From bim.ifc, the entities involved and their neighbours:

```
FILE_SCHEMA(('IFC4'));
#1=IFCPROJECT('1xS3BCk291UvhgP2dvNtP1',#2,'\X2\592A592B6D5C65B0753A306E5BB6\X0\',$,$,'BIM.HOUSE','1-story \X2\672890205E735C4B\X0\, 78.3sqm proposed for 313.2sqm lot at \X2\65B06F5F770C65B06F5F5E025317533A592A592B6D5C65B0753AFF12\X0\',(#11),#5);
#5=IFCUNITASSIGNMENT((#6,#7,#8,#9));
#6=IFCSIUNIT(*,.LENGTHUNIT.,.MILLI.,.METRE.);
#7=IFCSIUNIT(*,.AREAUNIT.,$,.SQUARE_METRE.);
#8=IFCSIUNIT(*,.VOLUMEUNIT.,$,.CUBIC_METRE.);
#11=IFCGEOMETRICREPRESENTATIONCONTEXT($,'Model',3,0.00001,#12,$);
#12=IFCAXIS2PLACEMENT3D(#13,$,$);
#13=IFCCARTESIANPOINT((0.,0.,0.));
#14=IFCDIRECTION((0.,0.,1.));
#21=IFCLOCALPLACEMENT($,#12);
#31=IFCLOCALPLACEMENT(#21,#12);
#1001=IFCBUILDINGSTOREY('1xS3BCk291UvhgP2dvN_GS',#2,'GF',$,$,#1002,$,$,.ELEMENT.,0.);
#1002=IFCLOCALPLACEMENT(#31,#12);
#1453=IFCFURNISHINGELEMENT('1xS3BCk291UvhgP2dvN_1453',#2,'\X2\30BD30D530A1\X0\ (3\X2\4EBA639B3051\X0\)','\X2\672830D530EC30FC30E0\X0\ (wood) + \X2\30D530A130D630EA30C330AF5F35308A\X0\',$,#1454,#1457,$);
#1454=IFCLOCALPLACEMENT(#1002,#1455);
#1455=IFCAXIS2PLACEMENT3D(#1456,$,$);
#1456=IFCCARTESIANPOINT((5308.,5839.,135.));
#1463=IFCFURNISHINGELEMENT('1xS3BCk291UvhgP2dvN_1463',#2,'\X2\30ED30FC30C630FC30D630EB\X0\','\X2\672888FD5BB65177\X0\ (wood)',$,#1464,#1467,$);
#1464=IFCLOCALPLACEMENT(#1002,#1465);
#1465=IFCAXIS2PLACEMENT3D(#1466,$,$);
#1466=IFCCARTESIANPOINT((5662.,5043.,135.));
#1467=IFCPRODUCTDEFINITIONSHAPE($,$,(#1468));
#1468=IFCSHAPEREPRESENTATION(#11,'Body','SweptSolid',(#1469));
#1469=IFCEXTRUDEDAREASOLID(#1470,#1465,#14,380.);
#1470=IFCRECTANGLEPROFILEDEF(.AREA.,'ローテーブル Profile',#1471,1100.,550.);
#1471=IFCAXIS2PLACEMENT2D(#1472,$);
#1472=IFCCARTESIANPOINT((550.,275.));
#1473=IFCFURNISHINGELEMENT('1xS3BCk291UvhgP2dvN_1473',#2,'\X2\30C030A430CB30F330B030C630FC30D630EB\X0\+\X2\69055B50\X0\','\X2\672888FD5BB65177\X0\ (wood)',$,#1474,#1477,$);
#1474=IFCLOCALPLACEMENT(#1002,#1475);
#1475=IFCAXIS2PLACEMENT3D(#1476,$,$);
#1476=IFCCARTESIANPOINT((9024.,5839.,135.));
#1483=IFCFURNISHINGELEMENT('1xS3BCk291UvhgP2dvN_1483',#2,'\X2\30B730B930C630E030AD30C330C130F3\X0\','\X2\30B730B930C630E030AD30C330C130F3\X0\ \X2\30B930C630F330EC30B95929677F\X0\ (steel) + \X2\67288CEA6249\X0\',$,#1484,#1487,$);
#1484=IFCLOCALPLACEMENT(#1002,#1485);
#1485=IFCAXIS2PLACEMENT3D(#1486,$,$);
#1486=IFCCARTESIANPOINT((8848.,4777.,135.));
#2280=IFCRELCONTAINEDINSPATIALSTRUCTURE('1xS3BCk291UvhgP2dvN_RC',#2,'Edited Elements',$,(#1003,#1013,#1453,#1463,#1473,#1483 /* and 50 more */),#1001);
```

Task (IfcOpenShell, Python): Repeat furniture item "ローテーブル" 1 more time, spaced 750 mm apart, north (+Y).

```python
import numpy as np
import ifcopenshell
import ifcopenshell.api.geometry
import ifcopenshell.api.root
import ifcopenshell.util.element
import ifcopenshell.util.placement
import ifcopenshell.util.unit

model = ifcopenshell.open("bim.ifc")
unit_scale = ifcopenshell.util.unit.calculate_unit_scale(model)


def reuse_history(source, copy):
    """copy_class also copies each property set's owner history, people and application; keep the originals."""
    for rel in copy.IsDefinedBy:
        if rel.is_a("IfcRelDefinesByProperties") and (history := rel.RelatingPropertyDefinition.OwnerHistory):
            rel.RelatingPropertyDefinition.OwnerHistory = source.OwnerHistory
            ifcopenshell.util.element.remove_deep2(model, history)


source = model.by_guid("1xS3BCk291UvhgP2dvN_1463")
base = ifcopenshell.util.placement.get_local_placement(source.ObjectPlacement)
step = np.array([0.0, 1.0, 0.0]) * 0.75 / unit_scale

for i in range(1, 2):
    copy = ifcopenshell.api.root.copy_class(model, product=source)
    copy.Representation = ifcopenshell.util.element.copy_deep(
        model, source.Representation, exclude=["IfcGeometricRepresentationContext", "IfcRepresentationMap"]
    )
    reuse_history(source, copy)
    matrix = base.copy()
    matrix[:3, 3] += i * step
    print("added at", matrix[:3, 3].round(3) + 0.0)
    ifcopenshell.api.geometry.edit_object_placement(model, product=copy, matrix=matrix, is_si=False)

model.write("bim_rev.ifc")
```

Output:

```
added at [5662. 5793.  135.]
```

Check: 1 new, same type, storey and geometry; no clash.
